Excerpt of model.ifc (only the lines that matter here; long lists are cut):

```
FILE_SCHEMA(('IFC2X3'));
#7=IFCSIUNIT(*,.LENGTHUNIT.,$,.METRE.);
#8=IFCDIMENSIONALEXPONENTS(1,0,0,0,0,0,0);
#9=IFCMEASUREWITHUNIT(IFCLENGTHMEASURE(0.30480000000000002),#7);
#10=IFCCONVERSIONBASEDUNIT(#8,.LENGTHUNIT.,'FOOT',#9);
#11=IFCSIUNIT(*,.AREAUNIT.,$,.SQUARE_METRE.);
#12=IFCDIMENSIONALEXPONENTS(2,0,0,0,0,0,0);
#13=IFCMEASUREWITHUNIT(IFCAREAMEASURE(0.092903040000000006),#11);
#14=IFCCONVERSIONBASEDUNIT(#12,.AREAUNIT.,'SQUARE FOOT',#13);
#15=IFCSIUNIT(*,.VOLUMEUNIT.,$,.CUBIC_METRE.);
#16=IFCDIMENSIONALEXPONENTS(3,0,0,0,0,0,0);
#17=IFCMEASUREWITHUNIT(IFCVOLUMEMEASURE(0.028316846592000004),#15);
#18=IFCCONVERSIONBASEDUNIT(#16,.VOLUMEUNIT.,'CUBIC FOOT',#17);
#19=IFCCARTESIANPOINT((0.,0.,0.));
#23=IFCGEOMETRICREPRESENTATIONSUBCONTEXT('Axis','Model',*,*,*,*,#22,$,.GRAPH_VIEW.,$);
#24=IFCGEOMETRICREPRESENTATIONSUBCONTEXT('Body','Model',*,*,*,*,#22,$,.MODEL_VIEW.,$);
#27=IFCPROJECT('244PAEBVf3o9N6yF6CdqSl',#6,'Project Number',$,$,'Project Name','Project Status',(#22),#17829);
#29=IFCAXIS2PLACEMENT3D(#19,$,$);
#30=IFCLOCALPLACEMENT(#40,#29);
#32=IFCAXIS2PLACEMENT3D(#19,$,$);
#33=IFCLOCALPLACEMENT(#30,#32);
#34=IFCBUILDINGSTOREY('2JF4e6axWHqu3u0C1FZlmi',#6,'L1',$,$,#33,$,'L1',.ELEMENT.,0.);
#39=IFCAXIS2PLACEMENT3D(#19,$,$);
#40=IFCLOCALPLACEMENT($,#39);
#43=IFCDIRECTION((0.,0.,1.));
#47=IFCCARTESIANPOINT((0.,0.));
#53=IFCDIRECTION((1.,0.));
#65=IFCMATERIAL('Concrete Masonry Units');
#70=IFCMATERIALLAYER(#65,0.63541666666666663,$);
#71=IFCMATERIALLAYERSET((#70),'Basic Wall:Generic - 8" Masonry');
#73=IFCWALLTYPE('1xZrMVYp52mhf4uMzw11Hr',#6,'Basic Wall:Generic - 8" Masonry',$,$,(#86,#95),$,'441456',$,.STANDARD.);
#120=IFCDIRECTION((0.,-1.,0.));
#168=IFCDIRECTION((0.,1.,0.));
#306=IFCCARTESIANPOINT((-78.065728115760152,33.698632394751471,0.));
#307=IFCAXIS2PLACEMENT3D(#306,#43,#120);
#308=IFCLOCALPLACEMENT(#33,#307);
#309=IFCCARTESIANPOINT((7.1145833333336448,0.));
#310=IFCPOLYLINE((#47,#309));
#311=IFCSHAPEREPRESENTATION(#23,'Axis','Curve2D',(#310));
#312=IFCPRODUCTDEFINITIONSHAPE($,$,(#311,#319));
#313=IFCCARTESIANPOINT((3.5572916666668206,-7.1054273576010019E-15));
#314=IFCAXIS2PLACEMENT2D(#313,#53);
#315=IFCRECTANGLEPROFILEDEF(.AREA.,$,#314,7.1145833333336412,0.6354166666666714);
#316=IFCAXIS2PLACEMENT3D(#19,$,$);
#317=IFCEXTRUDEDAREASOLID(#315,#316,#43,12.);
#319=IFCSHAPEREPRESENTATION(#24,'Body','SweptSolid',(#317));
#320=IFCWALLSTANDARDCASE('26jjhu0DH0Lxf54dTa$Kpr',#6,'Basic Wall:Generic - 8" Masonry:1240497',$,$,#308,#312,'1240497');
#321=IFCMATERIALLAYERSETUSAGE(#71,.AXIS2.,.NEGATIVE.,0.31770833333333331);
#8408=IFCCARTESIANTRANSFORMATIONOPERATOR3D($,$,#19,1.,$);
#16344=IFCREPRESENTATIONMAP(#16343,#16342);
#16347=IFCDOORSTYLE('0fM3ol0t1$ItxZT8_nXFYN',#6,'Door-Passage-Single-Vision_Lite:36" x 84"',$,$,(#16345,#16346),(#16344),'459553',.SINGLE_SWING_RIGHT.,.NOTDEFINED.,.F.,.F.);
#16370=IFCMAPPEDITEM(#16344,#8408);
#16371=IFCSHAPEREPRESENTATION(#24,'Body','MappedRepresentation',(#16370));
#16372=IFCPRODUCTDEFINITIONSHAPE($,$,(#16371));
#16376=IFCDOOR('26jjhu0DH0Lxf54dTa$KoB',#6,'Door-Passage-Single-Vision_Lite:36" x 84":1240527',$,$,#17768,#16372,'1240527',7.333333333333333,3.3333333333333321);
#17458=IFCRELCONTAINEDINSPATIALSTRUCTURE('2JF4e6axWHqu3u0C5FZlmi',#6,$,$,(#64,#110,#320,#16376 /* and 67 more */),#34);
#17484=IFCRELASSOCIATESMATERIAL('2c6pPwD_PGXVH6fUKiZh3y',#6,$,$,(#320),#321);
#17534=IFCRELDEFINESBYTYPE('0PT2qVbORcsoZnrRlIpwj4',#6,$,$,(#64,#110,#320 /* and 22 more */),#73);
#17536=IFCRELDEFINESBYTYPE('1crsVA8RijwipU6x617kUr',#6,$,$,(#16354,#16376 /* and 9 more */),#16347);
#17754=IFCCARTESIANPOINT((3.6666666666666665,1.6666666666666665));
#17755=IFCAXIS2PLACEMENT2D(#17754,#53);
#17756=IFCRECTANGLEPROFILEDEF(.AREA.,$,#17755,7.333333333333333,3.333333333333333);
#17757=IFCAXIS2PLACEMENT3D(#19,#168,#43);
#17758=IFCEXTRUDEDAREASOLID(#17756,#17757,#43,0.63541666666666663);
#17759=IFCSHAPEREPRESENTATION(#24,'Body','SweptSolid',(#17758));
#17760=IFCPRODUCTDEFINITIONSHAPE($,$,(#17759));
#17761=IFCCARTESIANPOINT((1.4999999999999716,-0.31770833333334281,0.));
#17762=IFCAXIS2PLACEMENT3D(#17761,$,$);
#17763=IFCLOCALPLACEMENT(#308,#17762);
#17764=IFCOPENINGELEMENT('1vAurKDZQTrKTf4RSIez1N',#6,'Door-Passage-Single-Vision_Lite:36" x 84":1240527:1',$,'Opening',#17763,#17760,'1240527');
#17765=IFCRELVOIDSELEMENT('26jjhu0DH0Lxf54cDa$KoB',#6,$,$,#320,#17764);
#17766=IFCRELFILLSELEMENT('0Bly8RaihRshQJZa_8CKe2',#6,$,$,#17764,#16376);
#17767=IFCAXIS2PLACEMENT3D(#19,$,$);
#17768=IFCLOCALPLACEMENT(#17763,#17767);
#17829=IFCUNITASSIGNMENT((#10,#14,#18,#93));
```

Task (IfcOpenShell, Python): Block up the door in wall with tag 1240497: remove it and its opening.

```python
import ifcopenshell
import ifcopenshell.api.feature
import ifcopenshell.api.root
import ifcopenshell.geom
import ifcopenshell.util.shape

model = ifcopenshell.open("model.ifc")
settings = ifcopenshell.geom.settings()


def volume(element):
    """Net volume in cubic metres, openings subtracted."""
    shape = ifcopenshell.geom.create_shape(settings, element)
    return ifcopenshell.util.shape.get_volume(shape.geometry)


door = model.by_id(16376)
opening = door.FillsVoids[0].RelatingOpeningElement
wall = opening.VoidsElements[0].RelatingBuildingElement
before = volume(wall)

ifcopenshell.api.root.remove_product(model, product=door)
ifcopenshell.api.feature.remove_feature(model, feature=opening)

after = volume(wall)

print(f"wall volume {before:.3f} -> {after:.3f} m3")

model.write("model_v2.ifc")
```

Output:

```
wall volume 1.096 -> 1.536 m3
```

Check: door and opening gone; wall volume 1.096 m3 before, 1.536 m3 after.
